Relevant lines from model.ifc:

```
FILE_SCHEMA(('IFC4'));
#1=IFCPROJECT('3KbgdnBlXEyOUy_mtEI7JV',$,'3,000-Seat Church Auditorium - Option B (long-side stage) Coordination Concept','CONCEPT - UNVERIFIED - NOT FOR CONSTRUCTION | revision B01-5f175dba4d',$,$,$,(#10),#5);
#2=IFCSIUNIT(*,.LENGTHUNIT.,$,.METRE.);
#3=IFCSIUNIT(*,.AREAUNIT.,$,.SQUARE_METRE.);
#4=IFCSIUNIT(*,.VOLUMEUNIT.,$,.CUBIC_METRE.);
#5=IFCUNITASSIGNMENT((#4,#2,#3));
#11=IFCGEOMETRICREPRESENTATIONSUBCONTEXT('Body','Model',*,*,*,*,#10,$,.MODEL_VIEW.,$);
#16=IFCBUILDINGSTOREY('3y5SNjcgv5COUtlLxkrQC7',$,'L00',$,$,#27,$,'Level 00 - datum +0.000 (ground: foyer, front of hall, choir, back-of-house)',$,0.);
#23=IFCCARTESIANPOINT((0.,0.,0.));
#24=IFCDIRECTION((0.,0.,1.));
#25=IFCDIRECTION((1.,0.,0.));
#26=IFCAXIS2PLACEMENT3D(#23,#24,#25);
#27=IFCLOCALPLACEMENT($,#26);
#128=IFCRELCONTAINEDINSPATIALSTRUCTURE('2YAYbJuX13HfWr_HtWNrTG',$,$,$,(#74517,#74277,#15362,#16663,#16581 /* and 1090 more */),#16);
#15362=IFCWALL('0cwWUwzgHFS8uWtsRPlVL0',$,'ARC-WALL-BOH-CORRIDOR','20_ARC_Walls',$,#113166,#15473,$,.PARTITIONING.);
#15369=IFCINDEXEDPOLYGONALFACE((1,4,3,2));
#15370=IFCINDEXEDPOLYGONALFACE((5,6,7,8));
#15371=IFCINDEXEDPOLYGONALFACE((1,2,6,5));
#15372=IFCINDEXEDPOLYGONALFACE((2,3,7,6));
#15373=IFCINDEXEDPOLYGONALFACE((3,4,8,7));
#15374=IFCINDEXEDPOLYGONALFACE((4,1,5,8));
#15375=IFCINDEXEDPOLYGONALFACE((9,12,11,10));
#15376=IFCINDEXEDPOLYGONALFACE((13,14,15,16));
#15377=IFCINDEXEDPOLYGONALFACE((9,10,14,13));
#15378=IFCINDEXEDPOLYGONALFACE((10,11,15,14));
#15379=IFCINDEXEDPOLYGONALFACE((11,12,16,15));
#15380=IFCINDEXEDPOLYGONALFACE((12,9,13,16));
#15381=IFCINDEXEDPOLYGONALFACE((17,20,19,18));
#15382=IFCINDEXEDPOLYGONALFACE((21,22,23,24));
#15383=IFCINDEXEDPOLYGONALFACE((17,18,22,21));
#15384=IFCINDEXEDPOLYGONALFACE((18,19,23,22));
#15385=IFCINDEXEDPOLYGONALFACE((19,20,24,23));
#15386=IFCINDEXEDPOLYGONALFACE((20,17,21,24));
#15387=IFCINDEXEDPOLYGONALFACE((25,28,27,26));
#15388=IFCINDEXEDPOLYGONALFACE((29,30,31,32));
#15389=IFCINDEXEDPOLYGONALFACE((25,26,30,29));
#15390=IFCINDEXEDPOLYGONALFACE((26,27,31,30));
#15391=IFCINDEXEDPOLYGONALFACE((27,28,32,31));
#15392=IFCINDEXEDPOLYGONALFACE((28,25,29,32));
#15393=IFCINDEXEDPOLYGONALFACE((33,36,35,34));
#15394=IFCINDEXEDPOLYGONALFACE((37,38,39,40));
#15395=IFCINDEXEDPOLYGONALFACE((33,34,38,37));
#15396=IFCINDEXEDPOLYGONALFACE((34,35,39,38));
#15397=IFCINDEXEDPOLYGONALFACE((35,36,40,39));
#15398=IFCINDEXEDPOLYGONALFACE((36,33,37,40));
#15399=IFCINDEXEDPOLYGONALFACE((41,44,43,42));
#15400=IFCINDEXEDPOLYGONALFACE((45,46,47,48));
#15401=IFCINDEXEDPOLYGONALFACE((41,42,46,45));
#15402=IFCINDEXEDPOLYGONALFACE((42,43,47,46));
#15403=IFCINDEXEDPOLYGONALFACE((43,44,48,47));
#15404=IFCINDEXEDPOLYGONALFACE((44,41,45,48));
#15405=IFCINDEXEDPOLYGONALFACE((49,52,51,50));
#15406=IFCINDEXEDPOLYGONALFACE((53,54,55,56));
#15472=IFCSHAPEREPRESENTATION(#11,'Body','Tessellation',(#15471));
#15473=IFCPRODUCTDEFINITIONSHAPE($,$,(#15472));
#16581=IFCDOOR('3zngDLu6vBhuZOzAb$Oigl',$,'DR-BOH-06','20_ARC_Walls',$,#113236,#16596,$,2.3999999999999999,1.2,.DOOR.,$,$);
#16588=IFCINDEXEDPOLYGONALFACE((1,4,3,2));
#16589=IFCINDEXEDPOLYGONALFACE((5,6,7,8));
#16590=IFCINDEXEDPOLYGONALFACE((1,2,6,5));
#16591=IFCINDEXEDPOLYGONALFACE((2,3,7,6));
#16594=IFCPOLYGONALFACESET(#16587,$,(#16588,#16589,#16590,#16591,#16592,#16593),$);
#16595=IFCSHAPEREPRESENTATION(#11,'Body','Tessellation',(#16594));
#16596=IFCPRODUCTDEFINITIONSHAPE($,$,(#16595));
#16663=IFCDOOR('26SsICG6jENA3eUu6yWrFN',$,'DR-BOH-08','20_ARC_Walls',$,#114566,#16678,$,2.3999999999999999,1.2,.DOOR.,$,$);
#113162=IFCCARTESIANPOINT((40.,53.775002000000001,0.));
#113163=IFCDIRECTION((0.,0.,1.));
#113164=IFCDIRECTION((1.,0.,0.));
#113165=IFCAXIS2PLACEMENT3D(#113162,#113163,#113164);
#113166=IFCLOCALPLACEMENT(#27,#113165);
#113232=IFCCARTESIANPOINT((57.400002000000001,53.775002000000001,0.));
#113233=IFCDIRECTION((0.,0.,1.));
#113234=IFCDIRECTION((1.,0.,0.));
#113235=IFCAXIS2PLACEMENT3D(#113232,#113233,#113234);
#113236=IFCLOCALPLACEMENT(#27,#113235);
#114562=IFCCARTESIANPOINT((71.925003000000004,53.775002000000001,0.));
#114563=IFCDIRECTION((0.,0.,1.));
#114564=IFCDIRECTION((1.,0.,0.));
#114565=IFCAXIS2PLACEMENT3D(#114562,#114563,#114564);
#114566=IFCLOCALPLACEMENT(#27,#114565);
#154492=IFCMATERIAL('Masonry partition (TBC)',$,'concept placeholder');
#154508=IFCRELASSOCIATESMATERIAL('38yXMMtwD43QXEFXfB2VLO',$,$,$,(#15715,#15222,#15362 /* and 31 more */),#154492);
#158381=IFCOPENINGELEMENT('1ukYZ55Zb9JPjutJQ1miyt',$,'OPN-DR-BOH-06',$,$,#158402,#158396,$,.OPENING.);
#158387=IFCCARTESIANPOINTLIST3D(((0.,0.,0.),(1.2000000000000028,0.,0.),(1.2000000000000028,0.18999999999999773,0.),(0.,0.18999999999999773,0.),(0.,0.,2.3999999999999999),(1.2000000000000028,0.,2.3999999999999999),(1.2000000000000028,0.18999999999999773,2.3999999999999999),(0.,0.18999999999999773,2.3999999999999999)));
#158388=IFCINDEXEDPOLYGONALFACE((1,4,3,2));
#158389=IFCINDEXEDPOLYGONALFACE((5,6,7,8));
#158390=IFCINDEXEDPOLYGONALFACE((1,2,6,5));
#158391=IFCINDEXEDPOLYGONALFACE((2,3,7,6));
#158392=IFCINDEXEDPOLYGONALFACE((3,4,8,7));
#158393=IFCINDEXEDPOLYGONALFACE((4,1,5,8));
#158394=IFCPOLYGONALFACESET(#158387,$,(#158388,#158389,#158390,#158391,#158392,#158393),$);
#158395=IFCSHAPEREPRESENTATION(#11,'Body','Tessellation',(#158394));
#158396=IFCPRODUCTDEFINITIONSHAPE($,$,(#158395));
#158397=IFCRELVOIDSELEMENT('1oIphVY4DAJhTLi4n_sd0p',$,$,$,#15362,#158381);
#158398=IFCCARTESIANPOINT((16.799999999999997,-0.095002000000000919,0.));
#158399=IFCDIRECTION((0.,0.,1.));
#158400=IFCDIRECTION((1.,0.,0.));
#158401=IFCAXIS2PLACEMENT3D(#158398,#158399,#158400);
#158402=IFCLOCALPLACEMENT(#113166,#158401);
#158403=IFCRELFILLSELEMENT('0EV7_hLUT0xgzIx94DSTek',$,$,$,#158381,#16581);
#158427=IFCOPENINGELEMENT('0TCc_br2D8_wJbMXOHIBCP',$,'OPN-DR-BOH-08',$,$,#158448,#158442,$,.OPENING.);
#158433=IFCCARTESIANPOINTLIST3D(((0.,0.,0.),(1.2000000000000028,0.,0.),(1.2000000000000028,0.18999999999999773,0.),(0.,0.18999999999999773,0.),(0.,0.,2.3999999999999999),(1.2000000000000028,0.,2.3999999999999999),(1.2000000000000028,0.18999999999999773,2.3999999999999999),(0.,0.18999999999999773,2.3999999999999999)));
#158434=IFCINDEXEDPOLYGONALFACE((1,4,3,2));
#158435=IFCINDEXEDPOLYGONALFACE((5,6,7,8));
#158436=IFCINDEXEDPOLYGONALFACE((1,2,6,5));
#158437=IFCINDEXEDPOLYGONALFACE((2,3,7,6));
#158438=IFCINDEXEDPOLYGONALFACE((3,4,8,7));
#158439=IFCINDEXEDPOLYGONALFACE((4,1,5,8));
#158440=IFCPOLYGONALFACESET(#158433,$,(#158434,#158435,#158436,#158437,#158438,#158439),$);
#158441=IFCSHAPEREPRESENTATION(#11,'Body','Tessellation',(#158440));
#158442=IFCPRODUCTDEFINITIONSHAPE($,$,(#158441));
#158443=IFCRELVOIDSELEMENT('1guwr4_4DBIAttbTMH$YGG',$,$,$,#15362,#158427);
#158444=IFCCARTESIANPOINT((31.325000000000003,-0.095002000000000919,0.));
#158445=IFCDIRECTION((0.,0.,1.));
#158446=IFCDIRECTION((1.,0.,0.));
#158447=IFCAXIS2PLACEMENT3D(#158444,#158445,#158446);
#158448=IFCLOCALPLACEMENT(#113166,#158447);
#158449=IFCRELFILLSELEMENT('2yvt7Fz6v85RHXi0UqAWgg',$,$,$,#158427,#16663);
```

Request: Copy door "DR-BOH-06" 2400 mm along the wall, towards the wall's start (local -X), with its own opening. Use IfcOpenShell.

```python
import ifcopenshell
import ifcopenshell.api.feature
import ifcopenshell.api.geometry
import ifcopenshell.api.root
import ifcopenshell.geom
import ifcopenshell.util.element
import ifcopenshell.util.placement
import ifcopenshell.util.shape
import ifcopenshell.util.unit

model = ifcopenshell.open("model.ifc")
unit_scale = ifcopenshell.util.unit.calculate_unit_scale(model)
settings = ifcopenshell.geom.settings()


def volume(element):
    """Net volume in cubic metres, openings subtracted."""
    shape = ifcopenshell.geom.create_shape(settings, element)
    return ifcopenshell.util.shape.get_volume(shape.geometry)


door = model.by_guid("3zngDLu6vBhuZOzAb$Oigl")
opening = door.FillsVoids[0].RelatingOpeningElement
wall = opening.VoidsElements[0].RelatingBuildingElement
before = volume(wall)
shift = ifcopenshell.util.placement.get_local_placement(wall.ObjectPlacement)[:3, 0] * -2.4 / unit_scale

# copy_class copies the void relationship, type, container and properties, but no geometry.
new_opening = ifcopenshell.api.root.copy_class(model, product=opening)
new_opening.Representation = ifcopenshell.util.element.copy_deep(
    model, opening.Representation, exclude=["IfcGeometricRepresentationContext", "IfcRepresentationMap"]
)
new_door = ifcopenshell.api.root.copy_class(model, product=door)
new_door.Representation = ifcopenshell.util.element.copy_deep(
    model, door.Representation, exclude=["IfcGeometricRepresentationContext", "IfcRepresentationMap"]
)
ifcopenshell.api.feature.add_filling(model, opening=new_opening, element=new_door)

for old, new in ((opening, new_opening), (door, new_door)):
    matrix = ifcopenshell.util.placement.get_local_placement(old.ObjectPlacement)
    matrix[:3, 3] += shift
    ifcopenshell.api.geometry.edit_object_placement(model, product=new, matrix=matrix, is_si=False)

after = volume(wall)

print(f"wall volume {before:.3f} -> {after:.3f} m3")

model.write("model_edited.ifc")
```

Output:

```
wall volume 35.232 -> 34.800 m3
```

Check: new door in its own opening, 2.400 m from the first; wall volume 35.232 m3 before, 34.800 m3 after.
